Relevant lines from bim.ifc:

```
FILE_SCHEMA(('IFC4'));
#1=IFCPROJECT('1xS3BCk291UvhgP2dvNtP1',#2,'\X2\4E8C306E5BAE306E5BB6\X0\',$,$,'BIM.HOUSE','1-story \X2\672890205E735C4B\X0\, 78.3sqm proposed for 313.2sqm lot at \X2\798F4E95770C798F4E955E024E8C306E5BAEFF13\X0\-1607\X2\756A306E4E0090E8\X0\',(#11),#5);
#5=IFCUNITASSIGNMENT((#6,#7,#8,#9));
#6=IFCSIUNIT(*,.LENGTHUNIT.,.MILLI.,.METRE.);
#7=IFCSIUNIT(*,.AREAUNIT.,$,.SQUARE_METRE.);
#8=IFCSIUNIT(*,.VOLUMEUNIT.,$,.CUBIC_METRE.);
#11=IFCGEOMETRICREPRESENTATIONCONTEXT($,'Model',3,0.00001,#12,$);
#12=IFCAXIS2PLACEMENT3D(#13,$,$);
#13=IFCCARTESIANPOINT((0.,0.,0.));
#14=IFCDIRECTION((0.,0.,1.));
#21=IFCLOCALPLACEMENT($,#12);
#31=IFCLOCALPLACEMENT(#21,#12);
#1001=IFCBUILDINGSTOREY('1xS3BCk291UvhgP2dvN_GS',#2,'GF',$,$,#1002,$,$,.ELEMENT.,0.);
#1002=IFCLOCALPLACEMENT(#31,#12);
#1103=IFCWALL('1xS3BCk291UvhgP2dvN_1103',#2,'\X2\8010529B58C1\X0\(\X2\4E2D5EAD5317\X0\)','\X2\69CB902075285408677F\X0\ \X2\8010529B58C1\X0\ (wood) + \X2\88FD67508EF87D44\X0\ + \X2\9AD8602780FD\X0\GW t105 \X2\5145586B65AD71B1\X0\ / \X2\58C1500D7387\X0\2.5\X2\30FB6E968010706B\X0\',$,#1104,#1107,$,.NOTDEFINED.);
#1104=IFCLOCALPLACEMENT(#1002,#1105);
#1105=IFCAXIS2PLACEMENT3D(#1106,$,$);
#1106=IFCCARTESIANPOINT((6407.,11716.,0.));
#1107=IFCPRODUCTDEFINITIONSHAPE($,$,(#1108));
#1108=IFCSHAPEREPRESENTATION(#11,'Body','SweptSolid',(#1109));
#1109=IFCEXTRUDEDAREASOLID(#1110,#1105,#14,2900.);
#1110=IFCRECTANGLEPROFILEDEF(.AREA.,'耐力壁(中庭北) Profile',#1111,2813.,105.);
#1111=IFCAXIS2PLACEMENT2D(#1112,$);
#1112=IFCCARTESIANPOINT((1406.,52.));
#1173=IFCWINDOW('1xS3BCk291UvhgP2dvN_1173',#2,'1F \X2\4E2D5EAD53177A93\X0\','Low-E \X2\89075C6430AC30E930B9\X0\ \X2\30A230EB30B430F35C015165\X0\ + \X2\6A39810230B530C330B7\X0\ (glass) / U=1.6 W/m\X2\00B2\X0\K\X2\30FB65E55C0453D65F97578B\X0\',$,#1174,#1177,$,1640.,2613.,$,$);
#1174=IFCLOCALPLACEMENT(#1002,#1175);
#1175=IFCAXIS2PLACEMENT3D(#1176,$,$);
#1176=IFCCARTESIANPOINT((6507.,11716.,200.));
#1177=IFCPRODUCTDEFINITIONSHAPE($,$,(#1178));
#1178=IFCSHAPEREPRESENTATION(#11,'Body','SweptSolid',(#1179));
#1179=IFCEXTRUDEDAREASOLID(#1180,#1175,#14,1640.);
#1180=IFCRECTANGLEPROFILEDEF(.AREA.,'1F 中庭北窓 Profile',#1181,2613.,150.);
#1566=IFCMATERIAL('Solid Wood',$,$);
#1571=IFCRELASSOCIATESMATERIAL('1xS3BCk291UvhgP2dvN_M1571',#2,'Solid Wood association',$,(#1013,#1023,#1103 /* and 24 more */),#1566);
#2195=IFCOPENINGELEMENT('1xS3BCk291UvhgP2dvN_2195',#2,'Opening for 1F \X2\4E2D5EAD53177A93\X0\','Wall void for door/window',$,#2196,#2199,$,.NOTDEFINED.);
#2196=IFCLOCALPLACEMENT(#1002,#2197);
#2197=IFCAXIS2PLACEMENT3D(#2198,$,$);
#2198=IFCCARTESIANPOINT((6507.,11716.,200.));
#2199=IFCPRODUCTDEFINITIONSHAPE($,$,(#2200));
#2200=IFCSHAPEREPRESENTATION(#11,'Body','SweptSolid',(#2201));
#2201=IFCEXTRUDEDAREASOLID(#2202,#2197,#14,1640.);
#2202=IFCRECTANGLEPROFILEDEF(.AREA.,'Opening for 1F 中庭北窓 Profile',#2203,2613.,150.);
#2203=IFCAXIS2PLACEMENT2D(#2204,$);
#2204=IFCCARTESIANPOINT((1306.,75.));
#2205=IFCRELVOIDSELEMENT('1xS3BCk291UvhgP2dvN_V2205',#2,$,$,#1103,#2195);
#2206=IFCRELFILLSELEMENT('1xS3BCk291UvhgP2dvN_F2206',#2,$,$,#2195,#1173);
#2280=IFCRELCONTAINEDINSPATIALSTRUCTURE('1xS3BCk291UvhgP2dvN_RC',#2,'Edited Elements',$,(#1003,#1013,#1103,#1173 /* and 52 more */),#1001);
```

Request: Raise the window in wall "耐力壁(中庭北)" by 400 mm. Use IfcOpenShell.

```python
import numpy as np
import ifcopenshell
import ifcopenshell.api.geometry
import ifcopenshell.util.placement
import ifcopenshell.util.unit

model = ifcopenshell.open("bim.ifc")
unit_scale = ifcopenshell.util.unit.calculate_unit_scale(model)

window = model.by_id(1173)
opening = window.FillsVoids[0].RelatingOpeningElement
dz = 0.4 / unit_scale

shift = np.array([0.0, 0.0, dz])
# The window is not placed relative to its opening, so move both.
for product in (opening, window):
    matrix = ifcopenshell.util.placement.get_local_placement(product.ObjectPlacement)
    matrix[:3, 3] += shift
    ifcopenshell.api.geometry.edit_object_placement(model, product=product, matrix=matrix, is_si=False)

print(f"moved by {dz * unit_scale:+.3f} m")

model.write("bim_v2.ifc")
```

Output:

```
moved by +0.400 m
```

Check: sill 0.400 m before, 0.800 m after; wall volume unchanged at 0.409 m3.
